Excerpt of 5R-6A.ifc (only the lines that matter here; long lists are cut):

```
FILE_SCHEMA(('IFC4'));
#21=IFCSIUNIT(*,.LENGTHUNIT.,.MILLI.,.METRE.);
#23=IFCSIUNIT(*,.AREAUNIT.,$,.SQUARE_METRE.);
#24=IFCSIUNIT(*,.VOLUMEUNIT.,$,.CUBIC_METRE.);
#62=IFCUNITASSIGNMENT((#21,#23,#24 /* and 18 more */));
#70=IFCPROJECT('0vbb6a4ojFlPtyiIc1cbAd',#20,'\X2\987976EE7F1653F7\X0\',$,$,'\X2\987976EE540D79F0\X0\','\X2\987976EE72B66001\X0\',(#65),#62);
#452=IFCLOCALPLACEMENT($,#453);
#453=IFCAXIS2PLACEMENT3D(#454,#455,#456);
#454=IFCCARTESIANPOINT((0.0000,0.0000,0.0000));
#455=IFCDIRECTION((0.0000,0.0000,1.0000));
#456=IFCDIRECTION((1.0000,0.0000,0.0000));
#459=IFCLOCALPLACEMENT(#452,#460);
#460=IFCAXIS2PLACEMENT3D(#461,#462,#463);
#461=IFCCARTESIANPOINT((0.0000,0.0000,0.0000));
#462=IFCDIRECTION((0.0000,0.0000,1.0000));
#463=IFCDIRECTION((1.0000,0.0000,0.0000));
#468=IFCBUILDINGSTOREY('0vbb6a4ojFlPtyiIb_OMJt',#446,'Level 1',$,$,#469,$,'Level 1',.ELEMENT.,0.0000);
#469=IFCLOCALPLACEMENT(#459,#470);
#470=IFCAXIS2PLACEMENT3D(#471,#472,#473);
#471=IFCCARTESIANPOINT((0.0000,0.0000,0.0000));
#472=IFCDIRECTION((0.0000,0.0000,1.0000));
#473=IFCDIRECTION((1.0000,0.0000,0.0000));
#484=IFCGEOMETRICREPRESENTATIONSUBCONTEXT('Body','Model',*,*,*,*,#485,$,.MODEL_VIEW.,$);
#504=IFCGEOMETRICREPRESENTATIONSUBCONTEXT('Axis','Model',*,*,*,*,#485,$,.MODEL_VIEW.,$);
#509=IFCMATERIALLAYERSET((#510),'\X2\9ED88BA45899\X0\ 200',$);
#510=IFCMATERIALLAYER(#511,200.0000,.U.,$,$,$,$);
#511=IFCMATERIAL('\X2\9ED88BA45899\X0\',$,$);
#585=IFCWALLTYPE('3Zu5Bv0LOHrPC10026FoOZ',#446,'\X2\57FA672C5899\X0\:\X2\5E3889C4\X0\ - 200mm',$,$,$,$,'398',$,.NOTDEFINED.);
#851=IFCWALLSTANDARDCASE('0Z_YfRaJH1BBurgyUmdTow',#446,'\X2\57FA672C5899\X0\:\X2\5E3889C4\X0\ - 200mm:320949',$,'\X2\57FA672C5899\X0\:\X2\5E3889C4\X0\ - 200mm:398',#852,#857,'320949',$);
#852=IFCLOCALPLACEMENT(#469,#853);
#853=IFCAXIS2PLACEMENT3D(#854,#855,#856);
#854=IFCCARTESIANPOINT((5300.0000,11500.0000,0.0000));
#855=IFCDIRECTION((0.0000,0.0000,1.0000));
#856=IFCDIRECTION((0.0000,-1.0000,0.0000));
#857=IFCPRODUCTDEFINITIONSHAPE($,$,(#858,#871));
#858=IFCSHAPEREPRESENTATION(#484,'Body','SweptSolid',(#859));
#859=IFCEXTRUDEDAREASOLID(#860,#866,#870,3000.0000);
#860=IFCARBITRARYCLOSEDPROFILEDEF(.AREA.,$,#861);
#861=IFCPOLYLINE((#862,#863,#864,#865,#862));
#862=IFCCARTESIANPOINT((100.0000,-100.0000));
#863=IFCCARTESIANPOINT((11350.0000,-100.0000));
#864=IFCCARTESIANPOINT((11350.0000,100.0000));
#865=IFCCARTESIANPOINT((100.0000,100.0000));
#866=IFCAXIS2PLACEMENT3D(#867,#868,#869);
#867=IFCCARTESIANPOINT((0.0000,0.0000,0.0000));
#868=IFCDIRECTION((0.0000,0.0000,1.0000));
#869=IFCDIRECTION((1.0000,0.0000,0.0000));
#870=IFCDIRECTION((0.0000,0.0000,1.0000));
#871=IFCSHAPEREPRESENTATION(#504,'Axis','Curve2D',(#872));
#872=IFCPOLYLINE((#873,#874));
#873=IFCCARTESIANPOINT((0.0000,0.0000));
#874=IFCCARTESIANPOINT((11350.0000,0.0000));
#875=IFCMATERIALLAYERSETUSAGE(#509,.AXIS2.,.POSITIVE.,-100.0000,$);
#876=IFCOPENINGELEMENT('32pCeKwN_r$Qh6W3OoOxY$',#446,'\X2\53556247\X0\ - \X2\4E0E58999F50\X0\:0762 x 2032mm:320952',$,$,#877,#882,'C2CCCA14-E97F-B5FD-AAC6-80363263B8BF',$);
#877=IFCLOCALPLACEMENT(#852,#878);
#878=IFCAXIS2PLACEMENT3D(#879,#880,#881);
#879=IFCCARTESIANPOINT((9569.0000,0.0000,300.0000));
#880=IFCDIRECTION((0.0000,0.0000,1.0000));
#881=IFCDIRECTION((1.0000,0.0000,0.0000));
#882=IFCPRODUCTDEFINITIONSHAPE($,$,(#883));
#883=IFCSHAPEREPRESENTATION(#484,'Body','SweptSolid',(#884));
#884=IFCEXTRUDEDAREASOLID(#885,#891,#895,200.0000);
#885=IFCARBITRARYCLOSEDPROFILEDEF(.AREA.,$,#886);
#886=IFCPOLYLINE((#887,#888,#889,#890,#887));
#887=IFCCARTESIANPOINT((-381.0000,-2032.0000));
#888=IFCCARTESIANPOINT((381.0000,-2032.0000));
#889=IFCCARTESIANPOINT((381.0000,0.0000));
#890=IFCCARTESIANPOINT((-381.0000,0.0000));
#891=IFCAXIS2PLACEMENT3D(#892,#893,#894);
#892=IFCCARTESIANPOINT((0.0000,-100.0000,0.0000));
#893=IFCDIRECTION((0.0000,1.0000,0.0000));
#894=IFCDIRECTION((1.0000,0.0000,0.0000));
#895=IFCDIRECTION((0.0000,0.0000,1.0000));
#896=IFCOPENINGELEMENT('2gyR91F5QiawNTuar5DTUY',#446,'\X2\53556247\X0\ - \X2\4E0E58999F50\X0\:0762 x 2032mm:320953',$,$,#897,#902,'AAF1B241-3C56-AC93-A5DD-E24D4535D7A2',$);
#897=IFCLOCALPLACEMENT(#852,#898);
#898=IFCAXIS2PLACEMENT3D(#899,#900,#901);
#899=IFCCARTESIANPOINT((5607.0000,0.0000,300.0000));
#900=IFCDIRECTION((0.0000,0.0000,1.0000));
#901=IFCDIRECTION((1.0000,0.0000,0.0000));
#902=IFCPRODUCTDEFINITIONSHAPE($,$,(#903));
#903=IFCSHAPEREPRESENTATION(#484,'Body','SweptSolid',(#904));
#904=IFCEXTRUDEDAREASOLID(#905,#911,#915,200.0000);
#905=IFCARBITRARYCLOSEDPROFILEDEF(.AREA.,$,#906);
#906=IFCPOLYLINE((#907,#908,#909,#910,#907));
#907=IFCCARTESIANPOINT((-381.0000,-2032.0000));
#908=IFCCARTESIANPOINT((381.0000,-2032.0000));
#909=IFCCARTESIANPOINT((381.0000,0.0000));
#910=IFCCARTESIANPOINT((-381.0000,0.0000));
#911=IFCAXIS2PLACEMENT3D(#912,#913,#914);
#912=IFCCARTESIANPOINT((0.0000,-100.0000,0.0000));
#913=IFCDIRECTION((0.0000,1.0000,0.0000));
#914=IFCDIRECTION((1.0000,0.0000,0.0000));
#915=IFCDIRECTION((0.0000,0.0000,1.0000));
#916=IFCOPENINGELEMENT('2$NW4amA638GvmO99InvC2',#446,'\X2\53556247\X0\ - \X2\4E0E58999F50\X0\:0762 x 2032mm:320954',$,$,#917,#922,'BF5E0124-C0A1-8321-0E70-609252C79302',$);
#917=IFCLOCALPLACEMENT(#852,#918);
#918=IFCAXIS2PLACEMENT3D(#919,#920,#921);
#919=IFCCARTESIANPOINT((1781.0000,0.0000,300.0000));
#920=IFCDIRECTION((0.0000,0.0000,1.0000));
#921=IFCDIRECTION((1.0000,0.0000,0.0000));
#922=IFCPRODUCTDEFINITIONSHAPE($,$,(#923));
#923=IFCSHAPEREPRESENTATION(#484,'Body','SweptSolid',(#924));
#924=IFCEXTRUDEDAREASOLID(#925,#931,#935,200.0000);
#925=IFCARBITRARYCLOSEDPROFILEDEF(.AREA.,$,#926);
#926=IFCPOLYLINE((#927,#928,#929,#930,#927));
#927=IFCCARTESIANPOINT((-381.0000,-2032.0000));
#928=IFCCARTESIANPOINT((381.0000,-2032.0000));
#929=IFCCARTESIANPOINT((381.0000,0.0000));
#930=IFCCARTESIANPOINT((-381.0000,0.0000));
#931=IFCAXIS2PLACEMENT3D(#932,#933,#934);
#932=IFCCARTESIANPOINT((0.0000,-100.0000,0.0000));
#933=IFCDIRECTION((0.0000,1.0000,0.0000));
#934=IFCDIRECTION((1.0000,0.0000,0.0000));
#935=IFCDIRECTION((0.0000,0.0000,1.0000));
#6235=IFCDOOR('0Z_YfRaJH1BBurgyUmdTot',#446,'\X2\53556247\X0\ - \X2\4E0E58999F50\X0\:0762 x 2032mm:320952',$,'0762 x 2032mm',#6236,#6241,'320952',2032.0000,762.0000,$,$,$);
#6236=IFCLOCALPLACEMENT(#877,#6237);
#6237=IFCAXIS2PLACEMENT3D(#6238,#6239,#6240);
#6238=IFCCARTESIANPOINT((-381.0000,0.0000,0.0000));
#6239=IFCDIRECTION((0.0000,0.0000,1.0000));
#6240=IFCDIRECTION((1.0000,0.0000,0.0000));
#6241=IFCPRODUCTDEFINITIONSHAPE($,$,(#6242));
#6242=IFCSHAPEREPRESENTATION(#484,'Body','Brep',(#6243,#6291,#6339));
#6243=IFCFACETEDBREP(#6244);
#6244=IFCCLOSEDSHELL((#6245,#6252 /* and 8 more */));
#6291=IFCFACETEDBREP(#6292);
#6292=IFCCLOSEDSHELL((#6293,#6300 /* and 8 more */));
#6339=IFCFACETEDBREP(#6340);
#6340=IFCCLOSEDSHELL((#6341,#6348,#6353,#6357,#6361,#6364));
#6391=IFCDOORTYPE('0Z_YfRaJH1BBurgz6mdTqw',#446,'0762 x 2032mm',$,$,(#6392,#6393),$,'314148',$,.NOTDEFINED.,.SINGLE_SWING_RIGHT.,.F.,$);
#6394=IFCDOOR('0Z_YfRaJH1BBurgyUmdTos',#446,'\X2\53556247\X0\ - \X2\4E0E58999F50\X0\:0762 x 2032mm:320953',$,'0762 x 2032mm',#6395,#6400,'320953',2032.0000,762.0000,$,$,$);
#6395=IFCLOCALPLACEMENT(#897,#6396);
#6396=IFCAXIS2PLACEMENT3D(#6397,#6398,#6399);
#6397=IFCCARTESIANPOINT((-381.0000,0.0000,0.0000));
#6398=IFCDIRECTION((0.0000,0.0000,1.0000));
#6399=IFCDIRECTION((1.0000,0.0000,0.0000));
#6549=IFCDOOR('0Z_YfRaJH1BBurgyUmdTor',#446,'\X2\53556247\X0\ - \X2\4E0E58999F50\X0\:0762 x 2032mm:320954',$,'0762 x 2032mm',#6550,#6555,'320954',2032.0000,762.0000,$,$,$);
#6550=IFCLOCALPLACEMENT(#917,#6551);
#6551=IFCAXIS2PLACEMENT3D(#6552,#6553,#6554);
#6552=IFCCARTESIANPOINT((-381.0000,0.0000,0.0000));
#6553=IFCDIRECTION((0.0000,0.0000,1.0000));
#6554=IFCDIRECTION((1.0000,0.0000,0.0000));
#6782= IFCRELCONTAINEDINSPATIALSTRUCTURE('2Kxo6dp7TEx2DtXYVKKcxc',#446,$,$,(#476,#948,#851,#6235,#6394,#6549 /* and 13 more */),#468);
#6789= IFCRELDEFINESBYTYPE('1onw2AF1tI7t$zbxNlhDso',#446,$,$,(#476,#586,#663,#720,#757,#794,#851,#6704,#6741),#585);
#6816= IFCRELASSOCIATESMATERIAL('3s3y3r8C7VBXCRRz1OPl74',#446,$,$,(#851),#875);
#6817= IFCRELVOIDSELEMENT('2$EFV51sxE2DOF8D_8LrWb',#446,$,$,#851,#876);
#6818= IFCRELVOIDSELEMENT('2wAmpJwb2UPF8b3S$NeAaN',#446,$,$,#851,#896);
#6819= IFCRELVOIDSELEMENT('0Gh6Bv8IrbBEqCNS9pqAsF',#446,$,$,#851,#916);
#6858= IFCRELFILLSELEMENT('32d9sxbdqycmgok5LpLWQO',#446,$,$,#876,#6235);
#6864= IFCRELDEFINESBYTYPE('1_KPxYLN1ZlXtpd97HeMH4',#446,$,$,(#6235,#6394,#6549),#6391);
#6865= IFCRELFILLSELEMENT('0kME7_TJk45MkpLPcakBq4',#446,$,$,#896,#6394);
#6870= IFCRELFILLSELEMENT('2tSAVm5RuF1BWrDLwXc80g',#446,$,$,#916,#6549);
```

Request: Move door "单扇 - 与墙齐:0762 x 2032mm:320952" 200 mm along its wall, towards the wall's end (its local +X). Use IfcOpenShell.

```python
import ifcopenshell
import ifcopenshell.api.geometry
import ifcopenshell.util.placement

model = ifcopenshell.open("5R-6A.ifc")

door = model.by_guid("0Z_YfRaJH1BBurgyUmdTot")
opening = door.FillsVoids[0].RelatingOpeningElement
wall = opening.VoidsElements[0].RelatingBuildingElement

wall_matrix = ifcopenshell.util.placement.get_local_placement(wall.ObjectPlacement)
shift = wall_matrix[:3, 0] * 200.0
before = ifcopenshell.util.placement.get_local_placement(door.ObjectPlacement)[:3, 3].copy()

# The door is placed relative to its opening, so it follows when the opening moves.
matrix = ifcopenshell.util.placement.get_local_placement(opening.ObjectPlacement)
matrix[:3, 3] += shift
ifcopenshell.api.geometry.edit_object_placement(
    model, product=opening, matrix=matrix, is_si=False, should_transform_children=True
)

after = ifcopenshell.util.placement.get_local_placement(door.ObjectPlacement)[:3, 3]
print("door moved by", (after - before).round(3) + 0.0)

model.write("5R-6A_edited.ifc")
```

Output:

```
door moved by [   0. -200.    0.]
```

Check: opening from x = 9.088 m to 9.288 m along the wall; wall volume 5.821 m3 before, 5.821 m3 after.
